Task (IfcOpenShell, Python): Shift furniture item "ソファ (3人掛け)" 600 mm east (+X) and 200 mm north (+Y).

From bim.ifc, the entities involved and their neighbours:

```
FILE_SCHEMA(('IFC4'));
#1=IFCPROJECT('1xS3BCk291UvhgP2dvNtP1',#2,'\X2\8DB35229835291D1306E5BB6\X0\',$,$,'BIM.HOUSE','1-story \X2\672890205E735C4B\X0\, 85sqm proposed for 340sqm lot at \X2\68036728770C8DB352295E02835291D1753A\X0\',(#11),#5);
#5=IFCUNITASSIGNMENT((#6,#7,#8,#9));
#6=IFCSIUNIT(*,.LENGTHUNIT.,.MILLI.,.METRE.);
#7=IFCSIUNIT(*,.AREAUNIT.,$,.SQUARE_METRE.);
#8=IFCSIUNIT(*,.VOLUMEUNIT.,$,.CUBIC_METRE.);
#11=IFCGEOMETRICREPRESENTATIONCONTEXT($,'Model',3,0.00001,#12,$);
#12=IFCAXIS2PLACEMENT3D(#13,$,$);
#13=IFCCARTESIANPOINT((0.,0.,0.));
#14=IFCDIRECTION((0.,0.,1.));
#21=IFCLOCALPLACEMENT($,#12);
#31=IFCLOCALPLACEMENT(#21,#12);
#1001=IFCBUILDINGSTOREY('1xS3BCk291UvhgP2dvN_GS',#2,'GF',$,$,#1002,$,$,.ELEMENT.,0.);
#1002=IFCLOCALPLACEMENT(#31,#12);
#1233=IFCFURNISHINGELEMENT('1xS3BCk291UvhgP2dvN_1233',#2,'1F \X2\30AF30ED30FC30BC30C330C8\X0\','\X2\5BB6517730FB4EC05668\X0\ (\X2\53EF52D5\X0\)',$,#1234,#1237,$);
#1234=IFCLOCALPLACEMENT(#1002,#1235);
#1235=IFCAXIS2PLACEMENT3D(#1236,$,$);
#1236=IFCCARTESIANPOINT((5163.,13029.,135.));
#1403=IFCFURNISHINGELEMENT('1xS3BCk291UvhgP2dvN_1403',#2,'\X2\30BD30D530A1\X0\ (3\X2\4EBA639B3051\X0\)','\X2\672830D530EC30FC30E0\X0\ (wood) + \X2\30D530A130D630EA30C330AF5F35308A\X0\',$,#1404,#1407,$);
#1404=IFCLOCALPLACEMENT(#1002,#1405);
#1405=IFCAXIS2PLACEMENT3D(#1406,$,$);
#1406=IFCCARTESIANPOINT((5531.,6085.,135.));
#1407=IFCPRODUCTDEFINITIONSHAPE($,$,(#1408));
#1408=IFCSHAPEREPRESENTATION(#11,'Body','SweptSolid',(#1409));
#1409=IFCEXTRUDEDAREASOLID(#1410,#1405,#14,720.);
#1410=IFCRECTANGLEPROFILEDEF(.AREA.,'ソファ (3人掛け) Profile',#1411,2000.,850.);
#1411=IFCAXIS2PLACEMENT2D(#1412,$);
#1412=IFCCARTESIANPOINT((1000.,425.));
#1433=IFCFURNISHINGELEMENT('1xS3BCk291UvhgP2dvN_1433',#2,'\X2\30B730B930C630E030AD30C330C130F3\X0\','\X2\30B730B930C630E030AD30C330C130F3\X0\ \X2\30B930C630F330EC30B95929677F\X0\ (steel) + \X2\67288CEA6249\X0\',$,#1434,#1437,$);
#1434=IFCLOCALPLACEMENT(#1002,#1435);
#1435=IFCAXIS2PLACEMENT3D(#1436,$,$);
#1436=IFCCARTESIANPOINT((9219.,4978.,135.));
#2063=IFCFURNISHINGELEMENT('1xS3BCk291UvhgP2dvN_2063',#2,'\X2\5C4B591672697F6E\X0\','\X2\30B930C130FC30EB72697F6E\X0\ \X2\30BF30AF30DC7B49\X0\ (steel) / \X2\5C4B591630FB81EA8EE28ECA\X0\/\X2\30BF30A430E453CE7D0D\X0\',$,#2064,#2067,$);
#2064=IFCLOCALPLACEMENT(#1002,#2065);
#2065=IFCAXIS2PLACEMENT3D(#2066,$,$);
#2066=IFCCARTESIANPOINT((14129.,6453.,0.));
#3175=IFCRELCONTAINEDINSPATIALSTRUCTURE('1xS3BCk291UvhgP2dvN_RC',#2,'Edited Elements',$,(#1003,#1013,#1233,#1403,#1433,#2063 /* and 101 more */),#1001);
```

```python
import ifcopenshell
import ifcopenshell.api.geometry
import ifcopenshell.util.placement

model = ifcopenshell.open("bim.ifc")

item = model.by_guid("1xS3BCk291UvhgP2dvN_1403")
matrix = ifcopenshell.util.placement.get_local_placement(item.ObjectPlacement)
matrix[0, 3] += 600.0
matrix[1, 3] += 200.0
ifcopenshell.api.geometry.edit_object_placement(model, product=item, matrix=matrix, is_si=False)

print(ifcopenshell.util.placement.get_local_placement(item.ObjectPlacement).round(3) + 0.0)

model.write("bim-out.ifc")
```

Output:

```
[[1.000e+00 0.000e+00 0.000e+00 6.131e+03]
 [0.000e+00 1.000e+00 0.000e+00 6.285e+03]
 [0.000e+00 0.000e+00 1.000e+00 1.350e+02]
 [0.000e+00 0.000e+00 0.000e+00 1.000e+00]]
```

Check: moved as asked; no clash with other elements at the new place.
